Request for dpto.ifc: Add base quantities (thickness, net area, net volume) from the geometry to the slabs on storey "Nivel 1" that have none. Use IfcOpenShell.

First a look at what the model holds.

```python
import ifcopenshell
import ifcopenshell.util.element
import ifcopenshell.util.unit

model = ifcopenshell.open("dpto.ifc")
print(model.schema)
for unit_type in ("LENGTHUNIT", "AREAUNIT", "VOLUMEUNIT"):
    print(unit_type, ifcopenshell.util.unit.calculate_unit_scale(model, unit_type))
storey = next(s for s in model.by_type("IfcBuildingStorey") if s.Name == "Nivel 1")
slabs = [e for e in ifcopenshell.util.element.get_decomposition(storey) if e.is_a("IfcSlab")]
for e in sorted(slabs, key=lambda e: e.id()):
    print(e.id(), e.is_a(), e.Name, list(ifcopenshell.util.element.get_psets(e, qtos_only=True)), sep=" | ")
```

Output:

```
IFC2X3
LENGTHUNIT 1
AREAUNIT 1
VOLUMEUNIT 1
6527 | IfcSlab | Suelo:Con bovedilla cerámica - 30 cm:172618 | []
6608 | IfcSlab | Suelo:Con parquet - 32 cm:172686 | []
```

```python
import ifcopenshell
import ifcopenshell.api.pset
import ifcopenshell.geom
import ifcopenshell.util.element
import ifcopenshell.util.shape
import ifcopenshell.util.unit

model = ifcopenshell.open("dpto.ifc")
unit_scale = ifcopenshell.util.unit.calculate_unit_scale(model)
area_scale = ifcopenshell.util.unit.calculate_unit_scale(model, "AREAUNIT")
volume_scale = ifcopenshell.util.unit.calculate_unit_scale(model, "VOLUMEUNIT")
settings = ifcopenshell.geom.settings()

storey = next(s for s in model.by_type("IfcBuildingStorey") if s.Name == "Nivel 1")
slabs = [e for e in ifcopenshell.util.element.get_decomposition(storey) if e.is_a("IfcSlab")]

for e in sorted(slabs, key=lambda e: e.id()):
    if ifcopenshell.util.element.get_psets(e, qtos_only=True, should_inherit=False):
        continue
    # Geometry comes back in metres, in the element's own axes.
    shape = ifcopenshell.geom.create_shape(settings, e)
    values = {
        "Width": ifcopenshell.util.shape.get_z(shape.geometry) / unit_scale,
        "NetArea": ifcopenshell.util.shape.get_footprint_area(shape.geometry) / area_scale,
        "NetVolume": ifcopenshell.util.shape.get_volume(shape.geometry) / volume_scale,
    }
    qto = ifcopenshell.api.pset.add_qto(model, product=e, name="BaseQuantities")
    ifcopenshell.api.pset.edit_qto(model, qto=qto, properties=values)
    print(e.id(), {k: round(v, 3) for k, v in values.items()})

model.write("dpto-out.ifc")
```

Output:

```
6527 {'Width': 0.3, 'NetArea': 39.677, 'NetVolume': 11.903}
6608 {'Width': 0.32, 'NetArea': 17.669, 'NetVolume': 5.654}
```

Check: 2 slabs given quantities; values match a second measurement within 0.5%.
